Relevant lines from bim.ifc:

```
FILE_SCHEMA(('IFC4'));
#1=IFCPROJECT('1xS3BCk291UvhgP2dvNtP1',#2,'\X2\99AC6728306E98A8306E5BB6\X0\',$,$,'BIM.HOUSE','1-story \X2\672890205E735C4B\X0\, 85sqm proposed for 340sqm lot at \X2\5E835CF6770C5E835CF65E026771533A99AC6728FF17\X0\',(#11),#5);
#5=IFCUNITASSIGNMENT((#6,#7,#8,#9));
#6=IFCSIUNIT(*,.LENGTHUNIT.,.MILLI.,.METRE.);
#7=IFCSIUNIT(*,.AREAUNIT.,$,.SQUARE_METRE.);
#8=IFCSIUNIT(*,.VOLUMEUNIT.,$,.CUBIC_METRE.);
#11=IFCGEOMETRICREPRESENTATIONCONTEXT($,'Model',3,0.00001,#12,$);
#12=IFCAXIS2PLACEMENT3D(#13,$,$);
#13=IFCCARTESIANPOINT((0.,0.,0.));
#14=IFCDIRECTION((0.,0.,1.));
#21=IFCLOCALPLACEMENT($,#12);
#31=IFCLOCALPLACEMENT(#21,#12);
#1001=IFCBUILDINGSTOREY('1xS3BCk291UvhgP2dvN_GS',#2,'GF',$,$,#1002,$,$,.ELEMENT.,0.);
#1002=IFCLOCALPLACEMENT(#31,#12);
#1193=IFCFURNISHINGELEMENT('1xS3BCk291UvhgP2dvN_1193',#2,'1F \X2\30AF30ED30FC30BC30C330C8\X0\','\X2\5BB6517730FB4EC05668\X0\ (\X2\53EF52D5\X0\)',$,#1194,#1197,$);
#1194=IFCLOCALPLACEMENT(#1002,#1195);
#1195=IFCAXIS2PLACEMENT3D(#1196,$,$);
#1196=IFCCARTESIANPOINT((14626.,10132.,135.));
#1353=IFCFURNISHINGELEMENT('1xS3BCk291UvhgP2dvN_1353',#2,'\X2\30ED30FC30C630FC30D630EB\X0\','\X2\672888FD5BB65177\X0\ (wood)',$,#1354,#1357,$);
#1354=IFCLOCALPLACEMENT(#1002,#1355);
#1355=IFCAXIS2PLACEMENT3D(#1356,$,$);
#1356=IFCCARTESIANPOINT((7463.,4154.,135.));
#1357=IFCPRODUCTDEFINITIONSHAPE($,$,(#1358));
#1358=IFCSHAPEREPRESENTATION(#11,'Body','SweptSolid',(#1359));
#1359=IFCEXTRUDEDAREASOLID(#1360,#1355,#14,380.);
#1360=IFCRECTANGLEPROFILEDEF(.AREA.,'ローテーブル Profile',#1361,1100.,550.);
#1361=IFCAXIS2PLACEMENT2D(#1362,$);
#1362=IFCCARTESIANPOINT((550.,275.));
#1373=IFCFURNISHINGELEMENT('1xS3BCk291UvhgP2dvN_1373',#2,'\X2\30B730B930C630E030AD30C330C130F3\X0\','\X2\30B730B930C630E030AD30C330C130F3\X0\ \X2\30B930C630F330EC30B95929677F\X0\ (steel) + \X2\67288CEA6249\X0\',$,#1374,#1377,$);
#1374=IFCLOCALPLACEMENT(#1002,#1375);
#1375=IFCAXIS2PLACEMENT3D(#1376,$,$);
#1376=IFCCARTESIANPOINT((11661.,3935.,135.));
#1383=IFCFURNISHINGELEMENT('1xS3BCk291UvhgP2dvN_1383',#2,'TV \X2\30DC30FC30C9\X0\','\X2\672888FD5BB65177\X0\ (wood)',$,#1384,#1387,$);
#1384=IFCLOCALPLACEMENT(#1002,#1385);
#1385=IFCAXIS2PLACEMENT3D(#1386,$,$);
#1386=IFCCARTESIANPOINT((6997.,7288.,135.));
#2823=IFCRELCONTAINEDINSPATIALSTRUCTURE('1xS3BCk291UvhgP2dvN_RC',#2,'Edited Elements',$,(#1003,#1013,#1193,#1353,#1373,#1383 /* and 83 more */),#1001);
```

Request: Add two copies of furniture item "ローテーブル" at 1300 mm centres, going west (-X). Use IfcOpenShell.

```python
import numpy as np
import ifcopenshell
import ifcopenshell.api.geometry
import ifcopenshell.api.root
import ifcopenshell.util.element
import ifcopenshell.util.placement
import ifcopenshell.util.unit

model = ifcopenshell.open("bim.ifc")
unit_scale = ifcopenshell.util.unit.calculate_unit_scale(model)


def reuse_history(source, copy):
    """copy_class also copies each property set's owner history, people and application; keep the originals."""
    for rel in copy.IsDefinedBy:
        if rel.is_a("IfcRelDefinesByProperties") and (history := rel.RelatingPropertyDefinition.OwnerHistory):
            rel.RelatingPropertyDefinition.OwnerHistory = source.OwnerHistory
            ifcopenshell.util.element.remove_deep2(model, history)


source = model.by_id(1353)
base = ifcopenshell.util.placement.get_local_placement(source.ObjectPlacement)
step = np.array([-1.0, 0.0, 0.0]) * 1.3 / unit_scale

for i in range(1, 3):
    copy = ifcopenshell.api.root.copy_class(model, product=source)
    copy.Representation = ifcopenshell.util.element.copy_deep(
        model, source.Representation, exclude=["IfcGeometricRepresentationContext", "IfcRepresentationMap"]
    )
    reuse_history(source, copy)
    matrix = base.copy()
    matrix[:3, 3] += i * step
    print("added at", matrix[:3, 3].round(3) + 0.0)
    ifcopenshell.api.geometry.edit_object_placement(model, product=copy, matrix=matrix, is_si=False)

model.write("bim-out.ifc")
```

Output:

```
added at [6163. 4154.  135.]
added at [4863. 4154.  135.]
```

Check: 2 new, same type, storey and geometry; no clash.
